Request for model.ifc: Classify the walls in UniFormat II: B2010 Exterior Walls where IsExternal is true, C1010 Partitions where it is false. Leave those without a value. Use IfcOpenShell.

First a look at what the model holds.

```python
import ifcopenshell
import ifcopenshell.util.element

model = ifcopenshell.open("model.ifc")
print(model.schema)
print("classifications:", [c.Name for c in model.by_type("IfcClassification")])
values = [ifcopenshell.util.element.get_pset(e, "Pset_WallCommon", "IsExternal") for e in model.by_type("IfcWall")]
for value in (True, False, None):
    print("IsExternal", value, values.count(value))
```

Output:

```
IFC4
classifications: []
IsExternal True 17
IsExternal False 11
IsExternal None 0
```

```python
import ifcopenshell
import ifcopenshell.api.classification
import ifcopenshell.util.element

model = ifcopenshell.open("model.ifc")

system = ifcopenshell.api.classification.add_classification(model, classification="UniFormat II")

walls = model.by_type("IfcWall")
external = {e: ifcopenshell.util.element.get_pset(e, "Pset_WallCommon", "IsExternal") for e in walls}
for flag, code, name in ((True, "B2010", "Exterior Walls"), (False, "C1010", "Partitions")):
    products = [e for e in walls if external[e] is flag]
    ifcopenshell.api.classification.add_reference(
        model, products=products, classification=system, identification=code, name=name
    )
    print(code, len(products))

model.write("model_edited.ifc")
```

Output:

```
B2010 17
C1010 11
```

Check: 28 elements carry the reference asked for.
